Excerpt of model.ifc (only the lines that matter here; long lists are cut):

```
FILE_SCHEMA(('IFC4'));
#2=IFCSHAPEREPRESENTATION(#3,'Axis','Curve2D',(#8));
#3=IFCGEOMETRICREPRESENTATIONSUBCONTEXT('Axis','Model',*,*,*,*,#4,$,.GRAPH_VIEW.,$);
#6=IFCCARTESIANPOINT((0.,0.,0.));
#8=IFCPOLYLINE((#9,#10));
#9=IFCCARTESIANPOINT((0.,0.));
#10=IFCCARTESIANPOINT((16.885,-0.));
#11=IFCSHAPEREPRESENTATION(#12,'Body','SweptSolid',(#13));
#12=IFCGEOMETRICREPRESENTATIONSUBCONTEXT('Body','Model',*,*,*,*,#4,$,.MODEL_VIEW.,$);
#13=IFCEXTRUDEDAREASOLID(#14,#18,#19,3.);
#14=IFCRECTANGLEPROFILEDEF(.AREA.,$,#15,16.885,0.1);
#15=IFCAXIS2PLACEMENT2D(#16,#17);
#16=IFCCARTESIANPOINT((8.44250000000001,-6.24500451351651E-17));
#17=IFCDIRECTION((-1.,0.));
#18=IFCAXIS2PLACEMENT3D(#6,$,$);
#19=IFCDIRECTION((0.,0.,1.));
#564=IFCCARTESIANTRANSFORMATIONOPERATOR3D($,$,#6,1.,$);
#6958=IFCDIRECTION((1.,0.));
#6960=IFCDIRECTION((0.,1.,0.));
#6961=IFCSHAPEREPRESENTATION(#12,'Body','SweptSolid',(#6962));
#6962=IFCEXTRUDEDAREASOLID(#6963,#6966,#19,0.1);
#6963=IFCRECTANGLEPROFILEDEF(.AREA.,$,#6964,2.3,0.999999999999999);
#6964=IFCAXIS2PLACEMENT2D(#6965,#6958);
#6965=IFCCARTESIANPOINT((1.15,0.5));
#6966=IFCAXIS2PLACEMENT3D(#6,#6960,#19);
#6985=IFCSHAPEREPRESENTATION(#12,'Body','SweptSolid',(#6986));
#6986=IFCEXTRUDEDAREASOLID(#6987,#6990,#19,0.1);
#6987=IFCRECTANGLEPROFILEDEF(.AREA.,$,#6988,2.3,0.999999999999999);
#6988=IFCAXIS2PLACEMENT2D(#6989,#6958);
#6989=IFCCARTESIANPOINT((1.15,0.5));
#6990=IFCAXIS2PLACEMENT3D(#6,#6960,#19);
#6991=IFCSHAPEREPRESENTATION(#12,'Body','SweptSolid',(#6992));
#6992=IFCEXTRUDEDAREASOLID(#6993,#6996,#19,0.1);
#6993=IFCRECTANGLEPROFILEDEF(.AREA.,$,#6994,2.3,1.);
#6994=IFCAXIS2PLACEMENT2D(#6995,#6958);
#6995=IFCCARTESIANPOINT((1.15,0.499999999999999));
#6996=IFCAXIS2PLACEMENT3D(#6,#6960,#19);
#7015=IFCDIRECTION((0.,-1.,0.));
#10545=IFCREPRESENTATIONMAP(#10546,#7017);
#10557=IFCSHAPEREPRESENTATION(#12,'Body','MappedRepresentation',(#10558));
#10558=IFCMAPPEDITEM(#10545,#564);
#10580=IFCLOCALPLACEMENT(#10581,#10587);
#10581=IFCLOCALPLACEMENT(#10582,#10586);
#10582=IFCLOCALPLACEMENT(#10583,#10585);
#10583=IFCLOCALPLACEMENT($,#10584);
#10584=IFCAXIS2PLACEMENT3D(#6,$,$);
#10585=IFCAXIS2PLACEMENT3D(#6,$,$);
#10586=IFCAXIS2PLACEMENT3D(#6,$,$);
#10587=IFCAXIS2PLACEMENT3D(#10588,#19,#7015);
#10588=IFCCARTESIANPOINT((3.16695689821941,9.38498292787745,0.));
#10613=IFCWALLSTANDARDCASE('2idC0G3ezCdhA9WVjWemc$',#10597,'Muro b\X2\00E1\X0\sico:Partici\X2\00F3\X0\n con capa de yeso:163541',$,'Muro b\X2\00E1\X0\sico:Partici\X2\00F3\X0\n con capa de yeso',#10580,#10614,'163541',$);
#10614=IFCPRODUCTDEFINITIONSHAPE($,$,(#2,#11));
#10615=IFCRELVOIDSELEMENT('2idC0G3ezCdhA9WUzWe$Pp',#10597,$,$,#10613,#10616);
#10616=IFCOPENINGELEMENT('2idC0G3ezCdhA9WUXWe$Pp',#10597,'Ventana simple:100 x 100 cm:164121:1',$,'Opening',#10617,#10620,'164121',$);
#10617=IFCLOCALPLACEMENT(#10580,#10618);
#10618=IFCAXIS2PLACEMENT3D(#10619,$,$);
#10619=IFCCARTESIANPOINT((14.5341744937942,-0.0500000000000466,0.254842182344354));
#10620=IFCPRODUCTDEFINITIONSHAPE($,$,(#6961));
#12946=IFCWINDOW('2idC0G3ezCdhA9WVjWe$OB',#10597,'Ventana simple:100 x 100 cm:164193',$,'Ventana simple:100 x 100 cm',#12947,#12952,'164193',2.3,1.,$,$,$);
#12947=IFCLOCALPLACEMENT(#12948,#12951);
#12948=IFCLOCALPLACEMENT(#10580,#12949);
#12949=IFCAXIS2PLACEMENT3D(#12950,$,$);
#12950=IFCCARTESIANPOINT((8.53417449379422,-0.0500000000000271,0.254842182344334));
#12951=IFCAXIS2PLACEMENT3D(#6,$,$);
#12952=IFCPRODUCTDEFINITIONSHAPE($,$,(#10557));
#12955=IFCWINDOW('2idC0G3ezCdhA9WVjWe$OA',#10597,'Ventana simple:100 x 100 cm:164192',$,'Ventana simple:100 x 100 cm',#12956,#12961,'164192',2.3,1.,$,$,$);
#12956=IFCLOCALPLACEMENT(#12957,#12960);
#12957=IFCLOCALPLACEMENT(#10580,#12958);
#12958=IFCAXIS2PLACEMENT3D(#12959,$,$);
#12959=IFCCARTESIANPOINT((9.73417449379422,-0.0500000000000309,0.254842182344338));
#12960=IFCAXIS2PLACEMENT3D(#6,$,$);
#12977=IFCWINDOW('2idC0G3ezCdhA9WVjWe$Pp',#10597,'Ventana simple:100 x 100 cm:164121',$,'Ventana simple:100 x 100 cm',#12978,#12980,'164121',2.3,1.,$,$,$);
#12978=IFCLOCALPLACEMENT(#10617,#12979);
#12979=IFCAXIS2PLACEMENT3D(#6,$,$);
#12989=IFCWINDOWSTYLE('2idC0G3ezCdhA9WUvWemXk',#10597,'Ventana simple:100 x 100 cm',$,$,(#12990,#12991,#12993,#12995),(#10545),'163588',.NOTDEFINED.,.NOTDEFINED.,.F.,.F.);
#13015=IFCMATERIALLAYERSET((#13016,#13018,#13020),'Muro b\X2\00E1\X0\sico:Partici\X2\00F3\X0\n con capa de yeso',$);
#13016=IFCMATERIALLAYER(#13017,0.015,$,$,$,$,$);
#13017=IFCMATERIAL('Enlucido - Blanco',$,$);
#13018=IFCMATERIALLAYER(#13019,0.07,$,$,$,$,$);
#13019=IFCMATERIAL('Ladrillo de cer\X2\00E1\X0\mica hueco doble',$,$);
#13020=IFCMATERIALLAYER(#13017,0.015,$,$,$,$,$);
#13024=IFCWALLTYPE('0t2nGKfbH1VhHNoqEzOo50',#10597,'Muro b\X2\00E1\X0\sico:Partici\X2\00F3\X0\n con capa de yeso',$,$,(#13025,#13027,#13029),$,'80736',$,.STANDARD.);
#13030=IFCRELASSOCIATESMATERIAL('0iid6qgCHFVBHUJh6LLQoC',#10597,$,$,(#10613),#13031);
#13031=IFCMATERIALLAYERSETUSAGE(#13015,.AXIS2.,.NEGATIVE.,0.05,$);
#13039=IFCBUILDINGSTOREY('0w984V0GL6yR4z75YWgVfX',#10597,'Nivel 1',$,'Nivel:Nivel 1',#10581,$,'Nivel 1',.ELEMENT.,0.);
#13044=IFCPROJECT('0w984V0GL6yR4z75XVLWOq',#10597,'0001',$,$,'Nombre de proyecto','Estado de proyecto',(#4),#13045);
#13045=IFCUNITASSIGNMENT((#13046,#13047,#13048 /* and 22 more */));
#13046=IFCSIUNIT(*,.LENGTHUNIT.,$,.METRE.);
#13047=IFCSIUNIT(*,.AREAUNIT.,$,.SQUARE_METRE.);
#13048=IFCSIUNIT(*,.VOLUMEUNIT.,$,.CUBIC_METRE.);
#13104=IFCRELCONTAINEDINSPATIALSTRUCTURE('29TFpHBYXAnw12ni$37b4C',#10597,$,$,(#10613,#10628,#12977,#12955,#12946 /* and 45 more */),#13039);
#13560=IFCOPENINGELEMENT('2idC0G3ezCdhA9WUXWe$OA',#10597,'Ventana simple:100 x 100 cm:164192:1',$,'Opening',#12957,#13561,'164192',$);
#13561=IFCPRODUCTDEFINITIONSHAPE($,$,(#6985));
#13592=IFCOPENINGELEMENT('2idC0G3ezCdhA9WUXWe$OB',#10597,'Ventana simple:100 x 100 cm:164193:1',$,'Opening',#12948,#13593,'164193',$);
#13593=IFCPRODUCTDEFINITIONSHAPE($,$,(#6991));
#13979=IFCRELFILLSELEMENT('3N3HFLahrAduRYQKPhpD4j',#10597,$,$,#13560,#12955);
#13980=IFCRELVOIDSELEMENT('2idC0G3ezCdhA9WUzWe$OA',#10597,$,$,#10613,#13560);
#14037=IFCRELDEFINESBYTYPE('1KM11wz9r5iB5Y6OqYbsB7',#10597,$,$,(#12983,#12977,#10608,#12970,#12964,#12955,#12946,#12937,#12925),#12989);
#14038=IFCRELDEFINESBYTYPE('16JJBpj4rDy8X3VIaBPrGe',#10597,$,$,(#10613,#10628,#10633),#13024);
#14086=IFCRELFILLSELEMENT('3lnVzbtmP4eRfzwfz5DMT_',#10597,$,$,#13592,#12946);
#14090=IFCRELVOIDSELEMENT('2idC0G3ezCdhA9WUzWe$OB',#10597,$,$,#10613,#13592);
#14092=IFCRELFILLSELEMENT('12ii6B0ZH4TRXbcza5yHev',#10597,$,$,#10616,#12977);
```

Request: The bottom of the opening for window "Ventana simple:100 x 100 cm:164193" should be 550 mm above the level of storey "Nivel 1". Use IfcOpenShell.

```python
import numpy as np
import ifcopenshell
import ifcopenshell.api.geometry
import ifcopenshell.geom
import ifcopenshell.util.element
import ifcopenshell.util.placement
import ifcopenshell.util.shape
import ifcopenshell.util.unit

model = ifcopenshell.open("model.ifc")
unit_scale = ifcopenshell.util.unit.calculate_unit_scale(model)

window = model.by_id(12946)
opening = window.FillsVoids[0].RelatingOpeningElement
storey = ifcopenshell.util.element.get_container(window, ifc_class="IfcBuildingStorey")
level = ifcopenshell.util.placement.get_local_placement(storey.ObjectPlacement)[2, 3]

# The opening's origin need not be at the sill, so measure its lowest point.
shape = ifcopenshell.geom.create_shape(ifcopenshell.geom.settings(), opening)
bottom = ifcopenshell.util.shape.get_shape_bottom_elevation(shape, shape.geometry) / unit_scale
dz = level + 0.55 - bottom

shift = np.array([0.0, 0.0, dz])
# The window is placed relative to its opening, so it follows when the opening moves.
matrix = ifcopenshell.util.placement.get_local_placement(opening.ObjectPlacement)
matrix[:3, 3] += shift
ifcopenshell.api.geometry.edit_object_placement(
    model, product=opening, matrix=matrix, is_si=False, should_transform_children=True
)

print(f"moved by {dz * unit_scale:+.3f} m")

model.write("model_edited.ifc")
```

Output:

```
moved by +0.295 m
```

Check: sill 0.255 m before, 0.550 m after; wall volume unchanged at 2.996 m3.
